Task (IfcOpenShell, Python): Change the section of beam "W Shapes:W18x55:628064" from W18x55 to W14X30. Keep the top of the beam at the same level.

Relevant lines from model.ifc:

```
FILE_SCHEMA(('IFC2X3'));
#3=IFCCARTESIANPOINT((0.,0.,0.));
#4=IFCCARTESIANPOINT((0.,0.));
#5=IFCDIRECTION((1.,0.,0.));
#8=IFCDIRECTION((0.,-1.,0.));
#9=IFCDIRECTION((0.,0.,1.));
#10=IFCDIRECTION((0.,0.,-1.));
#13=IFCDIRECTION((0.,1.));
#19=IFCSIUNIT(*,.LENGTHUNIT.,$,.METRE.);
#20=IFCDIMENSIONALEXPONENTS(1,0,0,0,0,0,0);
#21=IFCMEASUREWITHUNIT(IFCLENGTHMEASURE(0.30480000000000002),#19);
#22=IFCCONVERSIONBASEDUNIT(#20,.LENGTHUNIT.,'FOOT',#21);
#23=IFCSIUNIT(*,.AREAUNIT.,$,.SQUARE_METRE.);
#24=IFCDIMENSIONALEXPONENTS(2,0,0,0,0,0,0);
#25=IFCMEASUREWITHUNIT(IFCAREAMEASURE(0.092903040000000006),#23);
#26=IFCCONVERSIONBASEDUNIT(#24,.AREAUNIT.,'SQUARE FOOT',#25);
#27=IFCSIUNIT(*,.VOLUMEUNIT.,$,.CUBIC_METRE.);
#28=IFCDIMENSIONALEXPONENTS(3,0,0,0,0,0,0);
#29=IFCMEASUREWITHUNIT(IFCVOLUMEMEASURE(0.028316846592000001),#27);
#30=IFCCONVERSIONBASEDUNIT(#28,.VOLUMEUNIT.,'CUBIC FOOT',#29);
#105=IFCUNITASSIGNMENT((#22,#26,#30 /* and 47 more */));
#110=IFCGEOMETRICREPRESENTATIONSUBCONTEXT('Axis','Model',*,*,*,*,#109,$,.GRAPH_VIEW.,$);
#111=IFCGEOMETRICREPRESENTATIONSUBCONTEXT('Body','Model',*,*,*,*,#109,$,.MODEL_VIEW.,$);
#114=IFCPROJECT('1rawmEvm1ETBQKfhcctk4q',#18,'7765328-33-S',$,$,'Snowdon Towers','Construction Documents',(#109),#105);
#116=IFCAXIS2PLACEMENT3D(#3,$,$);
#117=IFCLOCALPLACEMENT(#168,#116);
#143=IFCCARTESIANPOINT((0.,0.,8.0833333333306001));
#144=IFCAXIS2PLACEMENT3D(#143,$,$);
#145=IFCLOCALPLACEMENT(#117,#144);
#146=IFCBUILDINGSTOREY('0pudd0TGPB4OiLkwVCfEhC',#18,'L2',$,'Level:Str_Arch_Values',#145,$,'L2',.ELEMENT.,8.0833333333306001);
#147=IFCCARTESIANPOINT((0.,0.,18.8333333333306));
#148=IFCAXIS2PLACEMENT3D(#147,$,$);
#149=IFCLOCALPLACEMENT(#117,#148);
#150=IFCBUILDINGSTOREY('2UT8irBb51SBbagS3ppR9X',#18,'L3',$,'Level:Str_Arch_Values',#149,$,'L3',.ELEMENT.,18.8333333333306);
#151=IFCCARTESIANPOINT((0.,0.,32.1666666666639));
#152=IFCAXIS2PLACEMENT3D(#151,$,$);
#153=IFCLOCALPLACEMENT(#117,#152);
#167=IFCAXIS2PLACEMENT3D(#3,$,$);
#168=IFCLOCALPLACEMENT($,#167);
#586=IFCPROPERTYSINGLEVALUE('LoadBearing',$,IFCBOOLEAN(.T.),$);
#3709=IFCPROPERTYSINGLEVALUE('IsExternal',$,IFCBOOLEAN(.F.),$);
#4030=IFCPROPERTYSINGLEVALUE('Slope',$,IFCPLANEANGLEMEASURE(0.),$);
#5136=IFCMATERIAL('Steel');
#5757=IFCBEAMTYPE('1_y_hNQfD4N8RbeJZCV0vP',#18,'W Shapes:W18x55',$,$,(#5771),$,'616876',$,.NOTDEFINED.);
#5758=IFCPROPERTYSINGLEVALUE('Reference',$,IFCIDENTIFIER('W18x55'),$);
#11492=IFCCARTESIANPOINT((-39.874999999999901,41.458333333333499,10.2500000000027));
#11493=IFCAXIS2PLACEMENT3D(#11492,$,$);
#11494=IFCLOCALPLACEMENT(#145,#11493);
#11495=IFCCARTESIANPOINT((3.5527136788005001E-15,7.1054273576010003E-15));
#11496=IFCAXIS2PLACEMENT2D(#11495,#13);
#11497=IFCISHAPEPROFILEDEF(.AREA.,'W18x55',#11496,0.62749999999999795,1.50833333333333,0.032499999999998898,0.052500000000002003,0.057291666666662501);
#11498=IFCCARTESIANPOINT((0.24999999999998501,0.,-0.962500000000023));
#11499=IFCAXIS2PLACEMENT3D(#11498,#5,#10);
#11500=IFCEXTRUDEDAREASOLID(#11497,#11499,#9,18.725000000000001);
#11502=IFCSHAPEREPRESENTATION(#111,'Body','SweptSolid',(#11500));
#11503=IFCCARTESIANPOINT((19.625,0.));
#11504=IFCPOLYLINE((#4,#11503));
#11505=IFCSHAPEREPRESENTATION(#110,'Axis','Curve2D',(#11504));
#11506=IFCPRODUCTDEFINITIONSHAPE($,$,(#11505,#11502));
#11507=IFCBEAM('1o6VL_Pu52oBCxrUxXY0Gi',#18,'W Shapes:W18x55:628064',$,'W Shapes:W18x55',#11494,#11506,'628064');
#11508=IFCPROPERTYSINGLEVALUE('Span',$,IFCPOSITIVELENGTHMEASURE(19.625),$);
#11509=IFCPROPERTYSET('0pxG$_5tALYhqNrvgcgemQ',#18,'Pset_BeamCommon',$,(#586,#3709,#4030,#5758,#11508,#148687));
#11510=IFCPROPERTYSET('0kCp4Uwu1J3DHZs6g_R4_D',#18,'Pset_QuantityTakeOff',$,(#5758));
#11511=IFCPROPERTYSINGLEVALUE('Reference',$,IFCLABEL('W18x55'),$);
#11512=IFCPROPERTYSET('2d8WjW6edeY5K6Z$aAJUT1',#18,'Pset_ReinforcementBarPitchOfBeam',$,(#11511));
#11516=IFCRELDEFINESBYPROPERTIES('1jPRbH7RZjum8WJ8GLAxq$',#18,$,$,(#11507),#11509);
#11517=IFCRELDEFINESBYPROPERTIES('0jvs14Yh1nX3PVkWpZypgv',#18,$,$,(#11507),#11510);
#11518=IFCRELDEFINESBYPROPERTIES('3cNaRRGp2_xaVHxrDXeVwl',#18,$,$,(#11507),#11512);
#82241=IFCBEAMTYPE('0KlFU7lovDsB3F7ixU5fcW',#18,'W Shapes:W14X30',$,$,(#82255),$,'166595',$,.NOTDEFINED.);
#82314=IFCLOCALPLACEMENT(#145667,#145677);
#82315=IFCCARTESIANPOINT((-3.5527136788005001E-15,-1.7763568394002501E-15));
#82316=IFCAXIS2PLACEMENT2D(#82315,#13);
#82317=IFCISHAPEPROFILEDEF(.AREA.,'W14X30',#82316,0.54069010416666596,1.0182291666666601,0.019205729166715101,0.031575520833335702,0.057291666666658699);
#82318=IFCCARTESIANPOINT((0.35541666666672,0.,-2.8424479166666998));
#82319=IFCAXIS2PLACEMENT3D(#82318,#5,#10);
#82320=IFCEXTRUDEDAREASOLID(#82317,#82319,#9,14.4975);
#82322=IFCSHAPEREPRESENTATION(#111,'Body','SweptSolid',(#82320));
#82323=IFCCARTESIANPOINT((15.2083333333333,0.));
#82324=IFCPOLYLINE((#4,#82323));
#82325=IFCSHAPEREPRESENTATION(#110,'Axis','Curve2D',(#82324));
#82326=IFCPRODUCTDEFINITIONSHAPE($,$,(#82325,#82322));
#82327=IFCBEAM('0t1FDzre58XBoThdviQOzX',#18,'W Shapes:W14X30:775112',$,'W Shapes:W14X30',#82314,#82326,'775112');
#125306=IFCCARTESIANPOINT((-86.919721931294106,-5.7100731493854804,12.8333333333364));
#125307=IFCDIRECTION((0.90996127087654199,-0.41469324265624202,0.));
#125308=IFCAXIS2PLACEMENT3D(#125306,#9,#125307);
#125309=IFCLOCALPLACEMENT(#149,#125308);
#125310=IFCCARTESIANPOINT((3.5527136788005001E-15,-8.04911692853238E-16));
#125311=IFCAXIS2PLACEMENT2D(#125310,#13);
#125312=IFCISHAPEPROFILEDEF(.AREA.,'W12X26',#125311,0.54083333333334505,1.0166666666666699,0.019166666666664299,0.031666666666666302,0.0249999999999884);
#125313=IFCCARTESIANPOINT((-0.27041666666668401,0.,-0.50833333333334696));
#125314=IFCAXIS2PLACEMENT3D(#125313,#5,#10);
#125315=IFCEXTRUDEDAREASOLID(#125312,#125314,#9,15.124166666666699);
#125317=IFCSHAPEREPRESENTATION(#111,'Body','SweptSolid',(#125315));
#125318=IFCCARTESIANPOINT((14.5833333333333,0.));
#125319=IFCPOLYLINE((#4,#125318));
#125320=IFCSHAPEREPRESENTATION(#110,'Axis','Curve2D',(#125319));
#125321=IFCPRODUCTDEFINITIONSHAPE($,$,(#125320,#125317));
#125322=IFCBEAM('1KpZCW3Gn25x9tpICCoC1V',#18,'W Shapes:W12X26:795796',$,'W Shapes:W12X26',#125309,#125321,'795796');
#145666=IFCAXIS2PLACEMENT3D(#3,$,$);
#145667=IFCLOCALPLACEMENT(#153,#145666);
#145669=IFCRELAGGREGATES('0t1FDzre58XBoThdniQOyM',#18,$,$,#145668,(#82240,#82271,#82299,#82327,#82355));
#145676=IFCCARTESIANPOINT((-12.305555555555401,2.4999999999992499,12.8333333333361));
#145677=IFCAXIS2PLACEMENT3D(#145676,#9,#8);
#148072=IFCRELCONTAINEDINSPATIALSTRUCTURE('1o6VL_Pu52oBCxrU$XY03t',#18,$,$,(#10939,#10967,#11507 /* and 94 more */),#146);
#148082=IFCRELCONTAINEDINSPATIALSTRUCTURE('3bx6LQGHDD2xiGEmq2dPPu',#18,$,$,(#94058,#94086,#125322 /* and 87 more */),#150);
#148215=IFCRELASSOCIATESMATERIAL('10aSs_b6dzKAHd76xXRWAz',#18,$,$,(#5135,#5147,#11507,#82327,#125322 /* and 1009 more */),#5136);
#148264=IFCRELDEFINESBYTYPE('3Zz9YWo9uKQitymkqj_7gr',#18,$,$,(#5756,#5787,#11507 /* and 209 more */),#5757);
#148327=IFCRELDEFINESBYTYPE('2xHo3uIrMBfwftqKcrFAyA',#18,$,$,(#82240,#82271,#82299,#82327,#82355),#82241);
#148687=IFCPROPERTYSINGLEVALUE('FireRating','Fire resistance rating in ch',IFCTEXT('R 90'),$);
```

```python
import ifcopenshell
import ifcopenshell.api.pset
import ifcopenshell.api.type
import ifcopenshell.util.element
import ifcopenshell.util.representation

model = ifcopenshell.open("model.ifc")

member = model.by_guid("1o6VL_Pu52oBCxrUxXY0Gi")
source = next(p for p in model.by_type("IfcIShapeProfileDef") if p.ProfileName == "W14X30")

body = ifcopenshell.util.representation.get_representation(member, "Model", "Body")
solid = body.Items[0]
old_profile = solid.SweptArea

# Copy the section's sizes but keep this member's own profile position.
profile = ifcopenshell.util.element.copy(model, source)
# Profiles are centred, so shift by half the change in depth to hold the top.
shift = (old_profile.OverallDepth - profile.OverallDepth) / 2
x, y = old_profile.Position.Location.Coordinates
up = (-1.0, 0.0)  # upwards, in the solid's own plane
location = model.createIfcCartesianPoint((x + up[0] * shift, y + up[1] * shift))
profile.Position = model.createIfcAxis2Placement2D(location, old_profile.Position.RefDirection)
solid.SweptArea = profile
if not model.get_total_inverses(old_profile):
    ifcopenshell.util.element.remove_deep2(model, old_profile)

new_type = model.by_guid("0KlFU7lovDsB3F7ixU5fcW")
ifcopenshell.api.type.assign_type(
    model, related_objects=[member], relating_type=new_type, should_map_representations=False
)
member.Name = member.Name.replace("W18x55", "W14X30")
member.ObjectType = "W Shapes:W14X30"
pset = model.by_id(ifcopenshell.util.element.get_pset(member, "Pset_BeamCommon", should_inherit=False)["id"])
ifcopenshell.api.pset.edit_pset(model, pset=pset, properties={"Reference": "W14X30"})
pset = model.by_id(ifcopenshell.util.element.get_pset(member, "Pset_QuantityTakeOff", should_inherit=False)["id"])
ifcopenshell.api.pset.edit_pset(model, pset=pset, properties={"Reference": "W14X30"})
pset = model.by_id(ifcopenshell.util.element.get_pset(member, "Pset_ReinforcementBarPitchOfBeam", should_inherit=False)["id"])
ifcopenshell.api.pset.edit_pset(model, pset=pset, properties={"Reference": "W14X30"})

print(solid.SweptArea)

model.write("model_rev.ifc")
```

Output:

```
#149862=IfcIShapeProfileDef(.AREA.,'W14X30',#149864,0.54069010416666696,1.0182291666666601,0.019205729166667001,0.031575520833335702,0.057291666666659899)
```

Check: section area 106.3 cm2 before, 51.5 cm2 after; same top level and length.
